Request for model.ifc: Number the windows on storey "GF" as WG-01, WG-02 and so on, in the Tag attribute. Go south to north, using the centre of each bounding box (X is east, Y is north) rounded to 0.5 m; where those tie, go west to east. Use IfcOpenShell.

First a look at what the model holds.

```python
import ifcopenshell
import ifcopenshell.util.element
import ifcopenshell.util.placement

model = ifcopenshell.open("model.ifc")
print(model.schema)
storey = next(s for s in model.by_type("IfcBuildingStorey") if s.Name == "GF")
windows = [e for e in ifcopenshell.util.element.get_decomposition(storey) if e.is_a("IfcWindow")]
for e in sorted(windows, key=lambda e: e.id()):
    origin = ifcopenshell.util.placement.get_local_placement(e.ObjectPlacement)[:3, 3]
    print(e.id(), e.Tag, e.Name, origin.round(2) + 0.0, sep=" | ")
```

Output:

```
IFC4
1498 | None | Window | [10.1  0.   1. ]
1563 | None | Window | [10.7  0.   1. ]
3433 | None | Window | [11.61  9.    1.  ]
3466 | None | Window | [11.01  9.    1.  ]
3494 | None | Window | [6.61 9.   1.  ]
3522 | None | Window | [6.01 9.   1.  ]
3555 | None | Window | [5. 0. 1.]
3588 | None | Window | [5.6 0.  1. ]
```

```python
import ifcopenshell
import ifcopenshell.geom
import ifcopenshell.util.element
import ifcopenshell.util.shape

model = ifcopenshell.open("model.ifc")
settings = ifcopenshell.geom.settings()
settings.set("use-world-coords", True)


def centre(element):
    shape = ifcopenshell.geom.create_shape(settings, element)
    return ifcopenshell.util.shape.get_bbox_centroid(shape.geometry)


storey = next(s for s in model.by_type("IfcBuildingStorey") if s.Name == "GF")
windows = [e for e in ifcopenshell.util.element.get_decomposition(storey) if e.is_a("IfcWindow")]

# Insertion points can sit at a corner or the storey origin, so sort by the geometry (in metres).
centres = {e: centre(e) for e in windows}
windows.sort(key=lambda e: (round(centres[e][1] / 0.5), centres[e][0]))

for i, e in enumerate(windows, start=1):
    number = f"WG-{i:02d}"
    e.Tag = number
    print(e.id(), number)

model.write("model_v2.ifc")
```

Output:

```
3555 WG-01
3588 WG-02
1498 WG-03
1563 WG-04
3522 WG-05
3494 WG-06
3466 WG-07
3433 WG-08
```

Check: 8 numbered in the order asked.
